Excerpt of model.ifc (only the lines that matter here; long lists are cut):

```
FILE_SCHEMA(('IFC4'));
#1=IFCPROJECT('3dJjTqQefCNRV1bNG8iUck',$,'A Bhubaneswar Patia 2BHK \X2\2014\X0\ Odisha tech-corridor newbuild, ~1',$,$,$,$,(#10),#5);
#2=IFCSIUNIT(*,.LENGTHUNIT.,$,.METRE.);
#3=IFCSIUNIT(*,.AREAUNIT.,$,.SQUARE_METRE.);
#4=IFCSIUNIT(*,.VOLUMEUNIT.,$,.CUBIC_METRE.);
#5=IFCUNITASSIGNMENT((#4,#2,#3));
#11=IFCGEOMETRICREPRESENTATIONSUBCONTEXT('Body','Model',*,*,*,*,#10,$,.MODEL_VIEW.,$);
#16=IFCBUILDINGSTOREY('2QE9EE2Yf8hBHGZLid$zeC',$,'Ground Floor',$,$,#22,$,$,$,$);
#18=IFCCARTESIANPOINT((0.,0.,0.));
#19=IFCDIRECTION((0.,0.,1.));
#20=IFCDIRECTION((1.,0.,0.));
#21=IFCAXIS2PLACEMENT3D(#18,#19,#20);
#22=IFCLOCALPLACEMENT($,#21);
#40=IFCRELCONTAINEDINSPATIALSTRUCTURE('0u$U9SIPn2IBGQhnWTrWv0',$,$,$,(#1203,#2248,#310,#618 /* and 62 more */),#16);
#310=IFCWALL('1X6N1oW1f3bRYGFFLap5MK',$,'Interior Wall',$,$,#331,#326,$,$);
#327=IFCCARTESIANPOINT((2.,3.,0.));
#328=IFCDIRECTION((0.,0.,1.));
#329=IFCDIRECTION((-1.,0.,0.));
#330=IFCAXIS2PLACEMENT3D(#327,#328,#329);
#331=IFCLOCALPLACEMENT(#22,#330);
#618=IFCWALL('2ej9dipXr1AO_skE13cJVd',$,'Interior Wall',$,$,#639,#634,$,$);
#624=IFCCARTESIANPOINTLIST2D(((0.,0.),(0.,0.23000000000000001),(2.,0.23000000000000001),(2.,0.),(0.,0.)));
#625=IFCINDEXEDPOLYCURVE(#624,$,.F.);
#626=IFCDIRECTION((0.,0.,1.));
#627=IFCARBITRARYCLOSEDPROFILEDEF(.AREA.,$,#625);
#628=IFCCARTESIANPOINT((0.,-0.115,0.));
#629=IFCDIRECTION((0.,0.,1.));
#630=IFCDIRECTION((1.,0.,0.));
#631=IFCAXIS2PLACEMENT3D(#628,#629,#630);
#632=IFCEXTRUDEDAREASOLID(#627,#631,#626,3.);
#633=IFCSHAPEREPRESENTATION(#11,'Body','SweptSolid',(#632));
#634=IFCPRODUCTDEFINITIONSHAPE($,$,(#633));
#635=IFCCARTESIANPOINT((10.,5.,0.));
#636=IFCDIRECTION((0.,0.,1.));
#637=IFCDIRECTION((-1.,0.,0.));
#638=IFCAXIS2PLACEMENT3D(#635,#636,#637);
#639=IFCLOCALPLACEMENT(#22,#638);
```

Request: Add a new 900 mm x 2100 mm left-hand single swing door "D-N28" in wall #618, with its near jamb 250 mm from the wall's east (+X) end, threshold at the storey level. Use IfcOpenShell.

```python
import numpy as np
import ifcopenshell
import ifcopenshell.api.feature
import ifcopenshell.api.geometry
import ifcopenshell.api.root
import ifcopenshell.api.spatial
import ifcopenshell.geom
import ifcopenshell.util.element
import ifcopenshell.util.placement
import ifcopenshell.util.representation
import ifcopenshell.util.shape
import ifcopenshell.util.unit

model = ifcopenshell.open("model.ifc")
unit_scale = ifcopenshell.util.unit.calculate_unit_scale(model)
settings = ifcopenshell.geom.settings()


def volume(element):
    """Net volume in cubic metres, openings subtracted."""
    shape = ifcopenshell.geom.create_shape(settings, element)
    return ifcopenshell.util.shape.get_volume(shape.geometry)


wall = model.by_id(618)
storey = ifcopenshell.util.element.get_container(wall, ifc_class="IfcBuildingStorey")
context = ifcopenshell.util.representation.get_context(model, "Model", "Body", "MODEL_VIEW")
before = volume(wall)

width, height, from_end, sill = 0.9, 2.1, 0.25, 0.0  # metres

# The wall runs along its own X axis, and the end named is its -X end.
wall_shape = ifcopenshell.geom.create_shape(settings, wall)
x, y, z = ifcopenshell.util.shape.get_vertices(wall_shape.geometry).T
start = x.min() + from_end
face, thickness = float(y.min()), float(y.max() - y.min())
wall_matrix = ifcopenshell.util.placement.get_local_placement(wall.ObjectPlacement)
level = ifcopenshell.util.placement.get_local_placement(storey.ObjectPlacement)[2, 3]


def in_wall(x, y):
    """Placement at x, y metres in the wall's axes, at sill height."""
    matrix = wall_matrix.copy()
    matrix[:, 3] = wall_matrix @ np.array([x / unit_scale, y / unit_scale, 0.0, 1.0])
    matrix[2, 3] = level + sill / unit_scale
    return matrix


# Opening: a box that overshoots both wall faces by 50 mm.
opening = ifcopenshell.api.root.create_entity(model, ifc_class="IfcOpeningElement", predefined_type="OPENING")
box = ifcopenshell.api.geometry.add_wall_representation(
    model, context=context, length=width, height=height, thickness=thickness + 0.1
)
ifcopenshell.api.geometry.assign_representation(model, product=opening, representation=box)
ifcopenshell.api.geometry.edit_object_placement(model, product=opening, matrix=in_wall(start, face - 0.05), is_si=False)
ifcopenshell.api.feature.add_feature(model, feature=opening, element=wall)

door = ifcopenshell.api.root.create_entity(model, ifc_class="IfcDoor", name="D-N28", predefined_type="DOOR")
door.OverallWidth, door.OverallHeight = width / unit_scale, height / unit_scale
door.OperationType = "SINGLE_SWING_LEFT"
body = ifcopenshell.api.geometry.add_door_representation(
    model,
    context=context,
    overall_width=door.OverallWidth,
    overall_height=door.OverallHeight,
    operation_type="SINGLE_SWING_LEFT",
    lining_properties={"LiningDepth": thickness / unit_scale, "ThresholdDepth": thickness / unit_scale},
)
ifcopenshell.api.geometry.assign_representation(model, product=door, representation=body)
ifcopenshell.api.spatial.assign_container(model, products=[door], relating_structure=storey)
ifcopenshell.api.feature.add_filling(model, opening=opening, element=door)

# The lining spans the wall, so the door starts at the wall face.
ifcopenshell.api.geometry.edit_object_placement(model, product=door, matrix=in_wall(start, face), is_si=False)

after = volume(wall)

print(f"wall volume {before:.3f} -> {after:.3f} m3")

model.write("model_updated.ifc")
```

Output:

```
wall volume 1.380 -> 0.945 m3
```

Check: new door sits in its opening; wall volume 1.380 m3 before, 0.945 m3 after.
